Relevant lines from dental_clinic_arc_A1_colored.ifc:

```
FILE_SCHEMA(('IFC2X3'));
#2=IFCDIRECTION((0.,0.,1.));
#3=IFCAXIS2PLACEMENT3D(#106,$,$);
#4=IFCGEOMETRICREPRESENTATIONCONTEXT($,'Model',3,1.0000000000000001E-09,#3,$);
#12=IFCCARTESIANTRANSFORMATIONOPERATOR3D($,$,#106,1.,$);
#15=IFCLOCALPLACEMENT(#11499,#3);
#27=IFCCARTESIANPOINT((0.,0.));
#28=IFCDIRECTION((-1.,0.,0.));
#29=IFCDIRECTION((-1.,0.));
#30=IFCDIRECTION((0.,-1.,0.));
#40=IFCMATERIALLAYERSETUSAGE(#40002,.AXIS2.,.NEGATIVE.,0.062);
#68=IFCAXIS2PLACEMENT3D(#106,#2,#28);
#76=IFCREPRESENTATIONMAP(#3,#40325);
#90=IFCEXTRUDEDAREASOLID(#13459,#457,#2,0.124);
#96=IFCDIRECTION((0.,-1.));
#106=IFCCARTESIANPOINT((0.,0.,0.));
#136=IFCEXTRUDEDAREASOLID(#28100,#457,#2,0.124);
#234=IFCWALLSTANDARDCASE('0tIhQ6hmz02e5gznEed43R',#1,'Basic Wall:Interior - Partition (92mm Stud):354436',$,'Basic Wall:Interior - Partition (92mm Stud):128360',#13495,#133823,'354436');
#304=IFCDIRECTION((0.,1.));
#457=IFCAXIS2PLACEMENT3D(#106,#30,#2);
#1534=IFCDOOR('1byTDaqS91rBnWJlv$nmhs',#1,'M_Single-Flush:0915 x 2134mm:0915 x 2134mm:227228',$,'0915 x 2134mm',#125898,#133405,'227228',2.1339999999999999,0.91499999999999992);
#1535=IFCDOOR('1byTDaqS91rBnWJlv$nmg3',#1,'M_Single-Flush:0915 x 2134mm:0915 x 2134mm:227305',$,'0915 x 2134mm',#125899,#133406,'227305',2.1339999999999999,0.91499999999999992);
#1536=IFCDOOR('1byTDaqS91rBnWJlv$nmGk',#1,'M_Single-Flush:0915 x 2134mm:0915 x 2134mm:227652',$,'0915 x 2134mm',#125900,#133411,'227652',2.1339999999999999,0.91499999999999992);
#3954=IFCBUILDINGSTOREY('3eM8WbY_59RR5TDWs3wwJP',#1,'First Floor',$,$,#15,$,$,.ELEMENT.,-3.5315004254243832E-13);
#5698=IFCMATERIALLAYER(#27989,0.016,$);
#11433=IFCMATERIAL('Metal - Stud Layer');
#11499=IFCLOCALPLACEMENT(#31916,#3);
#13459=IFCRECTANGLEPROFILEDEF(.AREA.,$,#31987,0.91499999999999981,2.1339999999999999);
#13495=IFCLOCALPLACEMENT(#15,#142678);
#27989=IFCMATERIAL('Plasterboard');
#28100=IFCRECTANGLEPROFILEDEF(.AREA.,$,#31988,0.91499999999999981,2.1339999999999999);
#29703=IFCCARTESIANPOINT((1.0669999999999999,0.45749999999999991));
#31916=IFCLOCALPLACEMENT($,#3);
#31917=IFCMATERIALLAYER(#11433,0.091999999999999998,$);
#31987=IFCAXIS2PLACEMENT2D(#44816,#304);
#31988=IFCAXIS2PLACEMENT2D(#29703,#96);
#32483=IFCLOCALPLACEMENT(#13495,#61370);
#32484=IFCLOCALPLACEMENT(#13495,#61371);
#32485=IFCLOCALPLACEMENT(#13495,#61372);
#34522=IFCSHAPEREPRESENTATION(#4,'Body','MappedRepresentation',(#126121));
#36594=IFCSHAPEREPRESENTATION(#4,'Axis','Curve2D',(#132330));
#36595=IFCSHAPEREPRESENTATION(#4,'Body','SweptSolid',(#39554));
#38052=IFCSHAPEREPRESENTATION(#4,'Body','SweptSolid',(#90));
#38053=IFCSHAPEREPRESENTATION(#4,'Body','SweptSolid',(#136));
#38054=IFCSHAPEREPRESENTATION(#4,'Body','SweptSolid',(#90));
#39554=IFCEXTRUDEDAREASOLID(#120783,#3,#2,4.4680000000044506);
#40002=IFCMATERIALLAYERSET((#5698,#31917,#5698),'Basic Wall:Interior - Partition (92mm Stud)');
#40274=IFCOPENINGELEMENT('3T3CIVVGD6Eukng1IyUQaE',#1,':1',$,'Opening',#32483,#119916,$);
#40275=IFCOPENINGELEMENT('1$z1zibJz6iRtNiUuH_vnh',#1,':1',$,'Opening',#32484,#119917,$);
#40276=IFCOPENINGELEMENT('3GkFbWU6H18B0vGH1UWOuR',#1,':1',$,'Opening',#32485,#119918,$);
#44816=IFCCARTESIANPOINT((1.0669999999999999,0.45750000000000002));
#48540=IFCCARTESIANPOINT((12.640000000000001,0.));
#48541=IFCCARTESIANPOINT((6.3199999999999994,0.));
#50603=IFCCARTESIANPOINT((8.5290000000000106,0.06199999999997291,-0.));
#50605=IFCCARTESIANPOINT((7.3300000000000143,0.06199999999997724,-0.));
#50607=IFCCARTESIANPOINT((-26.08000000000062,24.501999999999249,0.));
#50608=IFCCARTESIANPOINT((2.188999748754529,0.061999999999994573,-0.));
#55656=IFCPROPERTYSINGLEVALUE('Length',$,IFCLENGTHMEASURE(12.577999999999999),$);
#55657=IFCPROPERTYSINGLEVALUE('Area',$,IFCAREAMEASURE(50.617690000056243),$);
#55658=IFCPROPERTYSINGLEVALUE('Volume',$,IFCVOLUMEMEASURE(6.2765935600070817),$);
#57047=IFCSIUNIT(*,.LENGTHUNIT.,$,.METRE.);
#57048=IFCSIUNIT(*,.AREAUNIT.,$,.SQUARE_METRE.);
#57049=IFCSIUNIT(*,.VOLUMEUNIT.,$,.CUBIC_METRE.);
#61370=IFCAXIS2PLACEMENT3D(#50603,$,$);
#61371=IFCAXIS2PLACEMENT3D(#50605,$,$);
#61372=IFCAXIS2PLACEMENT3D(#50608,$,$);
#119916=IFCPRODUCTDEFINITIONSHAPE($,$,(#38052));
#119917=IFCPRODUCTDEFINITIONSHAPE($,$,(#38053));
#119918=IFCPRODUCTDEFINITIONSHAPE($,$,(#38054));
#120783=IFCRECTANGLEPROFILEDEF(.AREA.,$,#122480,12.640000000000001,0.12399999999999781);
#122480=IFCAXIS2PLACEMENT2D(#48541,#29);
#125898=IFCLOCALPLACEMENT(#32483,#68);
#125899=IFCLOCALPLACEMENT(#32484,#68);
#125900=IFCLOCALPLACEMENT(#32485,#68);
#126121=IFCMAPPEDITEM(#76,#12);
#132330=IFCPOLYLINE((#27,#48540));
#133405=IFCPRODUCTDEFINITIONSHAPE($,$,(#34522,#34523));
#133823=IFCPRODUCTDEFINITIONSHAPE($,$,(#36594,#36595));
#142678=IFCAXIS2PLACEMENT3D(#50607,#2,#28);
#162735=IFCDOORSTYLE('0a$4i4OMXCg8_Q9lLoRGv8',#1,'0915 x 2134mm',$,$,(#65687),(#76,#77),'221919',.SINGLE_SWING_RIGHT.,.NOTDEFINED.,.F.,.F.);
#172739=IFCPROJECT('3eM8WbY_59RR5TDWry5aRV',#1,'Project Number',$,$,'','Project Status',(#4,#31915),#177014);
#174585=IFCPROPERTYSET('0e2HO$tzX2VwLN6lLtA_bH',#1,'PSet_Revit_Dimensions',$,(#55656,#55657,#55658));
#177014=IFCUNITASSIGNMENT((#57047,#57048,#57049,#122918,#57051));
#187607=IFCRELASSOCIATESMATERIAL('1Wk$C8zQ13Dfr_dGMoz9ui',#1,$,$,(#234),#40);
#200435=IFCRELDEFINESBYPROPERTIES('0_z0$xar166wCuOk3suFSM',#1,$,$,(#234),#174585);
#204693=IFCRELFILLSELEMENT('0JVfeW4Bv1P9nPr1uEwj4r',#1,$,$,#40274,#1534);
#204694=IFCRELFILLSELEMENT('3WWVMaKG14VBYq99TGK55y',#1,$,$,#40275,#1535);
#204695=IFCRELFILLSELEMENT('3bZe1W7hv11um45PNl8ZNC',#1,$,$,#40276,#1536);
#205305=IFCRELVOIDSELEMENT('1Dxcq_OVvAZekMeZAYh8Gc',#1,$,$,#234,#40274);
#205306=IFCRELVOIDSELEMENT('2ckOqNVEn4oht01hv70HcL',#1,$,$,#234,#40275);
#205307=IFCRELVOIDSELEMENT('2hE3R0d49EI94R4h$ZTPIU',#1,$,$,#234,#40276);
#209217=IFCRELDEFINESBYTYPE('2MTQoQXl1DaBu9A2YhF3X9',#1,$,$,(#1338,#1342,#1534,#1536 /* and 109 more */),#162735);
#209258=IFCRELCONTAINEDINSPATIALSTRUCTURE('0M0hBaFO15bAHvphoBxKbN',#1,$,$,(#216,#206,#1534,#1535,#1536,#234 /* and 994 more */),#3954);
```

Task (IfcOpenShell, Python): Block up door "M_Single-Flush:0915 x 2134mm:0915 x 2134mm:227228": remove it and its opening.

```python
import ifcopenshell
import ifcopenshell.api.feature
import ifcopenshell.api.pset
import ifcopenshell.api.root
import ifcopenshell.geom
import ifcopenshell.util.element
import ifcopenshell.util.shape
import ifcopenshell.util.unit

model = ifcopenshell.open("dental_clinic_arc_A1_colored.ifc")
area_scale = ifcopenshell.util.unit.calculate_unit_scale(model, "AREAUNIT")
volume_scale = ifcopenshell.util.unit.calculate_unit_scale(model, "VOLUMEUNIT")
settings = ifcopenshell.geom.settings()


def volume(element):
    """Net volume in cubic metres, openings subtracted."""
    shape = ifcopenshell.geom.create_shape(settings, element)
    return ifcopenshell.util.shape.get_volume(shape.geometry)


door = model.by_guid("1byTDaqS91rBnWJlv$nmhs")
opening = door.FillsVoids[0].RelatingOpeningElement
wall = opening.VoidsElements[0].RelatingBuildingElement
before = volume(wall)

ifcopenshell.api.root.remove_product(model, product=door)
ifcopenshell.api.feature.remove_feature(model, feature=opening)

after = volume(wall)
thickness = 0.124  # wall thickness in metres

# Update the wall's stored quantities.
pset = model.by_id(ifcopenshell.util.element.get_pset(wall, "PSet_Revit_Dimensions", should_inherit=False)["id"])
ifcopenshell.api.pset.edit_pset(model, pset=pset, properties={
    "Area": model.create_entity("IfcAreaMeasure", after / thickness / area_scale),
    "Volume": model.create_entity("IfcVolumeMeasure", after / volume_scale),
})

print(f"wall volume {before:.3f} -> {after:.3f} m3")

model.write("dental_clinic_arc_A1_colored_rev.ifc")
```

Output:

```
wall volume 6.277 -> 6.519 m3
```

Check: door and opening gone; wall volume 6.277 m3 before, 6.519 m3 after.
